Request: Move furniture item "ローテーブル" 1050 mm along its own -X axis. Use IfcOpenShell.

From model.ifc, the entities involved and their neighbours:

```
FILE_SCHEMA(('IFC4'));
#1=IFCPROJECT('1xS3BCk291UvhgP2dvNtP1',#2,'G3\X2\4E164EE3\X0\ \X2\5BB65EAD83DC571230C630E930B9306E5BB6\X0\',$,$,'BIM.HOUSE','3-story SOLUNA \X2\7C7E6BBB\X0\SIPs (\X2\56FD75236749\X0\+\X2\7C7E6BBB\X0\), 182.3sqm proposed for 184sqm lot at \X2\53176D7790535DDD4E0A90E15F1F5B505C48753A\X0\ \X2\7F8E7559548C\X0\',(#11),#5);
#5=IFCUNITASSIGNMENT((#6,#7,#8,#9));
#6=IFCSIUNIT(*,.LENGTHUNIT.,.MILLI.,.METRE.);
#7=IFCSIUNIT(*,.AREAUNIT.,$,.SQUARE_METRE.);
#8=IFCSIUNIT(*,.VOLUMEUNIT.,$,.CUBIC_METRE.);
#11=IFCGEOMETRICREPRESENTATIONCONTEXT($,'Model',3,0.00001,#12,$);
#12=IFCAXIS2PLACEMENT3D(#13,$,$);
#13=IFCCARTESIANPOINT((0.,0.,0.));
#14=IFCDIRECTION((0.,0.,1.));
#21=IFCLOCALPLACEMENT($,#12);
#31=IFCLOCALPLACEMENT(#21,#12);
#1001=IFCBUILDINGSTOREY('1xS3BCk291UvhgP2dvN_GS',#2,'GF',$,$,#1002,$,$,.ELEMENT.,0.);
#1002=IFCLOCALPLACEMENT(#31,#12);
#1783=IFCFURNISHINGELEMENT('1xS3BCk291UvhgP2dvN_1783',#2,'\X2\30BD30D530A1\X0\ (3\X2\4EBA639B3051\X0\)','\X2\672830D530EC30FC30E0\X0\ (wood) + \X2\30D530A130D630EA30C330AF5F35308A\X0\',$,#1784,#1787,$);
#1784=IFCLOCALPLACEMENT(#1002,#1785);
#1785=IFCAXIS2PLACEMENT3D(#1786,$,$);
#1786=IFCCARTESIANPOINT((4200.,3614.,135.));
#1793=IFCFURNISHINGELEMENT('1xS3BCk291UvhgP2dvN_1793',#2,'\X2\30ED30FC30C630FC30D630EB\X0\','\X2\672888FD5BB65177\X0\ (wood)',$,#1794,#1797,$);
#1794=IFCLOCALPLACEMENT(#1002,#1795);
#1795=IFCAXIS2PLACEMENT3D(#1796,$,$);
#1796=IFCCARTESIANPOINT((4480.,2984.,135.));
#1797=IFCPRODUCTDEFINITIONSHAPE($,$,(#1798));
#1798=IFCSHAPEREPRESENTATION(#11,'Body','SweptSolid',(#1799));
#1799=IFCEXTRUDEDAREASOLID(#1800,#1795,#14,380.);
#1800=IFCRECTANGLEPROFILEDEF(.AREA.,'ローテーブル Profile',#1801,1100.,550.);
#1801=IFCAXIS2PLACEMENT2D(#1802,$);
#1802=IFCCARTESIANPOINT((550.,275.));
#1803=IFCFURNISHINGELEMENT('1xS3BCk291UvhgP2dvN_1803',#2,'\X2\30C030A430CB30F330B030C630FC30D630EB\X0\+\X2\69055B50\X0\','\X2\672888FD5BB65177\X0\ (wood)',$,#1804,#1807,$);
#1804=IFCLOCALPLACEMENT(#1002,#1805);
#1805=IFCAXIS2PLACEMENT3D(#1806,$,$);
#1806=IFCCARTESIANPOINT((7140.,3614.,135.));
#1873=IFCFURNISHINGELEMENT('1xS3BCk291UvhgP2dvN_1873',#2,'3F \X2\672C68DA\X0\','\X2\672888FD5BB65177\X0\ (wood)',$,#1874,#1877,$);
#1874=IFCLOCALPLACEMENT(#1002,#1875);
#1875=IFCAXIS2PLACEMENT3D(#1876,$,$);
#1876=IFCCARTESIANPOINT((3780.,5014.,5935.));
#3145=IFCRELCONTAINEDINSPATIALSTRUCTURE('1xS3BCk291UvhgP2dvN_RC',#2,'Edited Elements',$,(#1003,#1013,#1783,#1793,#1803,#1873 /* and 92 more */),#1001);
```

```python
import ifcopenshell
import ifcopenshell.api.geometry
import ifcopenshell.util.placement
import ifcopenshell.util.unit

model = ifcopenshell.open("model.ifc")
unit_scale = ifcopenshell.util.unit.calculate_unit_scale(model)

item = model.by_guid("1xS3BCk291UvhgP2dvN_1793")
matrix = ifcopenshell.util.placement.get_local_placement(item.ObjectPlacement)
matrix[:3, 3] -= matrix[:3, 0] * 1.05 / unit_scale
ifcopenshell.api.geometry.edit_object_placement(model, product=item, matrix=matrix, is_si=False)

print(ifcopenshell.util.placement.get_local_placement(item.ObjectPlacement).round(3) + 0.0)

model.write("model_edited.ifc")
```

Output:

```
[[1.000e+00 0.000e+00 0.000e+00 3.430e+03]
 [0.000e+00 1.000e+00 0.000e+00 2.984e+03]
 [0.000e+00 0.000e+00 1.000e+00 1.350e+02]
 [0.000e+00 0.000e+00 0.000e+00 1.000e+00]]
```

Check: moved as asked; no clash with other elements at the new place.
